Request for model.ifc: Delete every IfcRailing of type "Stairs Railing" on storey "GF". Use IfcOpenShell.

First a look at what the model holds.

```python
import ifcopenshell
import ifcopenshell.util.element

model = ifcopenshell.open("model.ifc")
print(model.schema)
storey = next(s for s in model.by_type("IfcBuildingStorey") if s.Name == "GF")
railings = [e for e in ifcopenshell.util.element.get_decomposition(storey) if e.is_a("IfcRailing")]
seen = {}
for e in railings:
    element_type = ifcopenshell.util.element.get_type(e)
    name = element_type.Name if element_type not in (None, e) else None
    seen[name] = seen.get(name, 0) + 1
for name, count in sorted(seen.items(), key=str):
    print(count, "x", name)
```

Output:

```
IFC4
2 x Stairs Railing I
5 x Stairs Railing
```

```python
import ifcopenshell
import ifcopenshell.api.root
import ifcopenshell.util.element

model = ifcopenshell.open("model.ifc")

storey = next(s for s in model.by_type("IfcBuildingStorey") if s.Name == "GF")
railings = [e for e in ifcopenshell.util.element.get_decomposition(storey) if e.is_a("IfcRailing")]
targets = [e for e in railings if (t := ifcopenshell.util.element.get_type(e)) not in (None, e) and t.Name == "Stairs Railing"]

for e in targets:
    ifcopenshell.api.root.remove_product(model, product=e)
print(len(targets), "removed")

model.write("model_v2.ifc")
```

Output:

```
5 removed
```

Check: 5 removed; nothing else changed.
